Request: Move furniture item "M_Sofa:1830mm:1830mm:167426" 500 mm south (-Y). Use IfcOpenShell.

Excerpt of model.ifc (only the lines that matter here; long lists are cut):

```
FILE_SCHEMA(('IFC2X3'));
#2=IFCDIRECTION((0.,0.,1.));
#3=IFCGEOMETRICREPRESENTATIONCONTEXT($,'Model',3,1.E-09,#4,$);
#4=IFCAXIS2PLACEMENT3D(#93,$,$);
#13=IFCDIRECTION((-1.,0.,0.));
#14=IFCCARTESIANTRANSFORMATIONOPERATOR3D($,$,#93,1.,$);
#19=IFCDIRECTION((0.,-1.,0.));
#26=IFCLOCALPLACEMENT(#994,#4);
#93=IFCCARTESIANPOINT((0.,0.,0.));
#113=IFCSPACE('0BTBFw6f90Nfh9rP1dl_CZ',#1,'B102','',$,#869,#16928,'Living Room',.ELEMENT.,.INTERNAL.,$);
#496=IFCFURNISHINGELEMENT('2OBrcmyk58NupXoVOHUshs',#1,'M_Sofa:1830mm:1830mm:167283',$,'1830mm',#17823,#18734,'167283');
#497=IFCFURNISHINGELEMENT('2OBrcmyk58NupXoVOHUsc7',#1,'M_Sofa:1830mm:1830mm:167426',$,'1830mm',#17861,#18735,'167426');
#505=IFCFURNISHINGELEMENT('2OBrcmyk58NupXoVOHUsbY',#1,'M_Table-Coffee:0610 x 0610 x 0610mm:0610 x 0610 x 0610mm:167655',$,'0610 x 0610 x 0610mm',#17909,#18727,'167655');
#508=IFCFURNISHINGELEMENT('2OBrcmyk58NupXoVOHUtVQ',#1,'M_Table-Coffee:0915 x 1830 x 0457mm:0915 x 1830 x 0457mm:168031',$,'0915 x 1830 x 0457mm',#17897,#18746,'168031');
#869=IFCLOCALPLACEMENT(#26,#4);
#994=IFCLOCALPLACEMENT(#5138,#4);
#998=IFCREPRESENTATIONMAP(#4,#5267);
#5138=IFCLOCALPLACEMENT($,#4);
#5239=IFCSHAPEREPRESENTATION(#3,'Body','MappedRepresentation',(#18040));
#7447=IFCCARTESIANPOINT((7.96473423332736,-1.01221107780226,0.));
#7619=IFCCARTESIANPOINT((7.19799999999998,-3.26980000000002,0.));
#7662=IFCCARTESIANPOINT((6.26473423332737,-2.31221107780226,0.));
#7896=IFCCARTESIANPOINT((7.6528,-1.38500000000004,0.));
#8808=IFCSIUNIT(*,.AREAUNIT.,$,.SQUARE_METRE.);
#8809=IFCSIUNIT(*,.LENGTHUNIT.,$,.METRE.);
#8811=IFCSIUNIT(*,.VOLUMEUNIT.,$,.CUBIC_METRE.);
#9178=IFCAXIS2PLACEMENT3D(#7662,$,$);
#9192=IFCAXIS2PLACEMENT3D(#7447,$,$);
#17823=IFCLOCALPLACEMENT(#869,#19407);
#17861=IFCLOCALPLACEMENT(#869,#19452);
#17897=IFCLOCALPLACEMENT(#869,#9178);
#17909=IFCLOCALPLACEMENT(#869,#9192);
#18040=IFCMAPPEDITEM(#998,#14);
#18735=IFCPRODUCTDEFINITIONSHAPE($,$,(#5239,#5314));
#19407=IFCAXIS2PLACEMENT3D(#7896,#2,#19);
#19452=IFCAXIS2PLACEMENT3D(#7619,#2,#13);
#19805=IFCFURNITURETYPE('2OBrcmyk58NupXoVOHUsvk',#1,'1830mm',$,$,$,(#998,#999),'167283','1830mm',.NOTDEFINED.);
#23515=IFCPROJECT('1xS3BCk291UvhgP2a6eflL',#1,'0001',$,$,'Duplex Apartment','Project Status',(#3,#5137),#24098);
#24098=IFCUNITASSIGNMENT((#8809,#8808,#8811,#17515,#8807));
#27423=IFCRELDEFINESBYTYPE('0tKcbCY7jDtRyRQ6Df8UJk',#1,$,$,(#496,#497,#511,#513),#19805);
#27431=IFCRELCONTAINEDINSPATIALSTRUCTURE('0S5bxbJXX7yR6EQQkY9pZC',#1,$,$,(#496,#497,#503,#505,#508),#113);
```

```python
import ifcopenshell
import ifcopenshell.api.geometry
import ifcopenshell.util.placement
import ifcopenshell.util.unit

model = ifcopenshell.open("model.ifc")
unit_scale = ifcopenshell.util.unit.calculate_unit_scale(model)

item = model.by_guid("2OBrcmyk58NupXoVOHUsc7")
matrix = ifcopenshell.util.placement.get_local_placement(item.ObjectPlacement)
matrix[1, 3] -= 0.5 / unit_scale
ifcopenshell.api.geometry.edit_object_placement(model, product=item, matrix=matrix, is_si=False)

print(ifcopenshell.util.placement.get_local_placement(item.ObjectPlacement).round(3) + 0.0)

model.write("model_updated.ifc")
```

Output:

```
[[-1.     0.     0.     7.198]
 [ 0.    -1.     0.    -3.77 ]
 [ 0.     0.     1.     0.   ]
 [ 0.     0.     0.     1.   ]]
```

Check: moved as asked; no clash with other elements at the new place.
